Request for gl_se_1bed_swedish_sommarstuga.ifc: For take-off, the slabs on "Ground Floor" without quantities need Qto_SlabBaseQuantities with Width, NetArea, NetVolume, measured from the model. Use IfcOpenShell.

First a look at what the model holds.

```python
import ifcopenshell
import ifcopenshell.util.element
import ifcopenshell.util.unit

model = ifcopenshell.open("gl_se_1bed_swedish_sommarstuga.ifc")
print(model.schema)
for unit_type in ("LENGTHUNIT", "AREAUNIT", "VOLUMEUNIT"):
    print(unit_type, ifcopenshell.util.unit.calculate_unit_scale(model, unit_type))
storey = next(s for s in model.by_type("IfcBuildingStorey") if s.Name == "Ground Floor")
slabs = [e for e in ifcopenshell.util.element.get_decomposition(storey) if e.is_a("IfcSlab")]
for e in sorted(slabs, key=lambda e: e.id()):
    print(e.id(), e.is_a(), e.Name, list(ifcopenshell.util.element.get_psets(e, qtos_only=True)), sep=" | ")
```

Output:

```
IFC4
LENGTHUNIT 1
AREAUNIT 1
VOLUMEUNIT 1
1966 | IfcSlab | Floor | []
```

```python
import ifcopenshell
import ifcopenshell.api.pset
import ifcopenshell.geom
import ifcopenshell.util.element
import ifcopenshell.util.shape
import ifcopenshell.util.unit

model = ifcopenshell.open("gl_se_1bed_swedish_sommarstuga.ifc")
unit_scale = ifcopenshell.util.unit.calculate_unit_scale(model)
area_scale = ifcopenshell.util.unit.calculate_unit_scale(model, "AREAUNIT")
volume_scale = ifcopenshell.util.unit.calculate_unit_scale(model, "VOLUMEUNIT")
settings = ifcopenshell.geom.settings()

storey = next(s for s in model.by_type("IfcBuildingStorey") if s.Name == "Ground Floor")
slabs = [e for e in ifcopenshell.util.element.get_decomposition(storey) if e.is_a("IfcSlab")]

for e in sorted(slabs, key=lambda e: e.id()):
    if ifcopenshell.util.element.get_psets(e, qtos_only=True, should_inherit=False):
        continue
    # Geometry comes back in metres, in the element's own axes.
    shape = ifcopenshell.geom.create_shape(settings, e)
    values = {
        "Width": ifcopenshell.util.shape.get_z(shape.geometry) / unit_scale,
        "NetArea": ifcopenshell.util.shape.get_footprint_area(shape.geometry) / area_scale,
        "NetVolume": ifcopenshell.util.shape.get_volume(shape.geometry) / volume_scale,
    }
    qto = ifcopenshell.api.pset.add_qto(model, product=e, name="Qto_SlabBaseQuantities")
    ifcopenshell.api.pset.edit_qto(model, qto=qto, properties=values)
    print(e.id(), {k: round(v, 3) for k, v in values.items()})

model.write("gl_se_1bed_swedish_sommarstuga_rev.ifc")
```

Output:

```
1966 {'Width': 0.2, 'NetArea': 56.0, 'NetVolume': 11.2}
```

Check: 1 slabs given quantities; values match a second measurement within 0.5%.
